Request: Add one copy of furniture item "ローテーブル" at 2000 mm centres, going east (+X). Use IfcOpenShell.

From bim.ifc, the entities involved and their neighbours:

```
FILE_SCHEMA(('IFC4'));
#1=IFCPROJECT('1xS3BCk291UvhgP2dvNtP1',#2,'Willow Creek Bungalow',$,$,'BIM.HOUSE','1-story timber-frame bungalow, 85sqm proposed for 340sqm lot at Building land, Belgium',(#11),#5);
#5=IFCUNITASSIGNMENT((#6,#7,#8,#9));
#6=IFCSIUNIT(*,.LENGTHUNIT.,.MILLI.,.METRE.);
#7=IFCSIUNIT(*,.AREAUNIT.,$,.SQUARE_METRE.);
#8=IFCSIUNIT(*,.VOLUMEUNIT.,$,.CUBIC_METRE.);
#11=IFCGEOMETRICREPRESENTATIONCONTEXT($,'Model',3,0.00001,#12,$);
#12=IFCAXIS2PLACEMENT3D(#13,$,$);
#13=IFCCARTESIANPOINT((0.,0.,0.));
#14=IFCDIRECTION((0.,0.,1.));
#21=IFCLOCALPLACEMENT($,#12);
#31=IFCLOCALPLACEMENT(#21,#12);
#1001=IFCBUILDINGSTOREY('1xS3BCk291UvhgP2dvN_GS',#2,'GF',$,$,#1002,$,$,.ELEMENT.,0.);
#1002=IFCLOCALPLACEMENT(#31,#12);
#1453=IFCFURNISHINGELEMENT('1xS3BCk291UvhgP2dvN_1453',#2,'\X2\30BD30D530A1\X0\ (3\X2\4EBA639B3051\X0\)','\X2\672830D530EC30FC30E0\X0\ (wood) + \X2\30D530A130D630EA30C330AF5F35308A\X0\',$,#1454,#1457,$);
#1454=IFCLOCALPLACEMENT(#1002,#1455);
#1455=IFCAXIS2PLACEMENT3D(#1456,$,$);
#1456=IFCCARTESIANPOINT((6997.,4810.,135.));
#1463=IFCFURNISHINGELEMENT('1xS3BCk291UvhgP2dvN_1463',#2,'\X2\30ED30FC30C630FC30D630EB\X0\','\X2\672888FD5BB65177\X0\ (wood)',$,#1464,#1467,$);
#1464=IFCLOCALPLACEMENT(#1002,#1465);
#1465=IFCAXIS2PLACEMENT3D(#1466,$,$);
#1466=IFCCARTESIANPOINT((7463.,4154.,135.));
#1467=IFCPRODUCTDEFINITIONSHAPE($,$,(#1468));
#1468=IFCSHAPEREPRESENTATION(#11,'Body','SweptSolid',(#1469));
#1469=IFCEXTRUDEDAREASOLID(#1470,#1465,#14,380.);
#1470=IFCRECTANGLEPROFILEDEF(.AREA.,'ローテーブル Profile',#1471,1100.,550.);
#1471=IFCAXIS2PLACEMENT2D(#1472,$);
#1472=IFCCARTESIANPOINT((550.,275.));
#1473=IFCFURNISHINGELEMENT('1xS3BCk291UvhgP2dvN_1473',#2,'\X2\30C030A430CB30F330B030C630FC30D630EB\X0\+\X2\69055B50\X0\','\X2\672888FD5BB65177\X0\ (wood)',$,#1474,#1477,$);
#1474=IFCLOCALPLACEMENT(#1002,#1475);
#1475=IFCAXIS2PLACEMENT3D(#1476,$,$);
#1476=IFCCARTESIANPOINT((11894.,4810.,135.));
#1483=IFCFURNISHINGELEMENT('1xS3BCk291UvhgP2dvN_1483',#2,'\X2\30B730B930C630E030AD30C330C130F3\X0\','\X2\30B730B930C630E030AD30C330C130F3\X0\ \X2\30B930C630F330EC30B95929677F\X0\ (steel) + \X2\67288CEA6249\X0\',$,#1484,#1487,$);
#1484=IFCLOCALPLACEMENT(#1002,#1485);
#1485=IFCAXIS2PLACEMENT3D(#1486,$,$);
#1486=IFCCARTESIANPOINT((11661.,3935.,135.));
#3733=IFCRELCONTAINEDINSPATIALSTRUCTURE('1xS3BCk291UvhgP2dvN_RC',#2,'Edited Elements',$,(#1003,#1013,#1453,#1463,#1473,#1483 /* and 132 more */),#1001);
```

```python
import numpy as np
import ifcopenshell
import ifcopenshell.api.geometry
import ifcopenshell.api.root
import ifcopenshell.util.element
import ifcopenshell.util.placement

model = ifcopenshell.open("bim.ifc")


def reuse_history(source, copy):
    """copy_class also copies each property set's owner history, people and application; keep the originals."""
    for rel in copy.IsDefinedBy:
        if rel.is_a("IfcRelDefinesByProperties") and (history := rel.RelatingPropertyDefinition.OwnerHistory):
            rel.RelatingPropertyDefinition.OwnerHistory = source.OwnerHistory
            ifcopenshell.util.element.remove_deep2(model, history)


source = model.by_guid("1xS3BCk291UvhgP2dvN_1463")
base = ifcopenshell.util.placement.get_local_placement(source.ObjectPlacement)
step = np.array([1.0, 0.0, 0.0]) * 2000.0

for i in range(1, 2):
    copy = ifcopenshell.api.root.copy_class(model, product=source)
    copy.Representation = ifcopenshell.util.element.copy_deep(
        model, source.Representation, exclude=["IfcGeometricRepresentationContext", "IfcRepresentationMap"]
    )
    reuse_history(source, copy)
    matrix = base.copy()
    matrix[:3, 3] += i * step
    print("added at", matrix[:3, 3].round(3) + 0.0)
    ifcopenshell.api.geometry.edit_object_placement(model, product=copy, matrix=matrix, is_si=False)

model.write("bim_rev.ifc")
```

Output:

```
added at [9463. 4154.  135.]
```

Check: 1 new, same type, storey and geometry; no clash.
